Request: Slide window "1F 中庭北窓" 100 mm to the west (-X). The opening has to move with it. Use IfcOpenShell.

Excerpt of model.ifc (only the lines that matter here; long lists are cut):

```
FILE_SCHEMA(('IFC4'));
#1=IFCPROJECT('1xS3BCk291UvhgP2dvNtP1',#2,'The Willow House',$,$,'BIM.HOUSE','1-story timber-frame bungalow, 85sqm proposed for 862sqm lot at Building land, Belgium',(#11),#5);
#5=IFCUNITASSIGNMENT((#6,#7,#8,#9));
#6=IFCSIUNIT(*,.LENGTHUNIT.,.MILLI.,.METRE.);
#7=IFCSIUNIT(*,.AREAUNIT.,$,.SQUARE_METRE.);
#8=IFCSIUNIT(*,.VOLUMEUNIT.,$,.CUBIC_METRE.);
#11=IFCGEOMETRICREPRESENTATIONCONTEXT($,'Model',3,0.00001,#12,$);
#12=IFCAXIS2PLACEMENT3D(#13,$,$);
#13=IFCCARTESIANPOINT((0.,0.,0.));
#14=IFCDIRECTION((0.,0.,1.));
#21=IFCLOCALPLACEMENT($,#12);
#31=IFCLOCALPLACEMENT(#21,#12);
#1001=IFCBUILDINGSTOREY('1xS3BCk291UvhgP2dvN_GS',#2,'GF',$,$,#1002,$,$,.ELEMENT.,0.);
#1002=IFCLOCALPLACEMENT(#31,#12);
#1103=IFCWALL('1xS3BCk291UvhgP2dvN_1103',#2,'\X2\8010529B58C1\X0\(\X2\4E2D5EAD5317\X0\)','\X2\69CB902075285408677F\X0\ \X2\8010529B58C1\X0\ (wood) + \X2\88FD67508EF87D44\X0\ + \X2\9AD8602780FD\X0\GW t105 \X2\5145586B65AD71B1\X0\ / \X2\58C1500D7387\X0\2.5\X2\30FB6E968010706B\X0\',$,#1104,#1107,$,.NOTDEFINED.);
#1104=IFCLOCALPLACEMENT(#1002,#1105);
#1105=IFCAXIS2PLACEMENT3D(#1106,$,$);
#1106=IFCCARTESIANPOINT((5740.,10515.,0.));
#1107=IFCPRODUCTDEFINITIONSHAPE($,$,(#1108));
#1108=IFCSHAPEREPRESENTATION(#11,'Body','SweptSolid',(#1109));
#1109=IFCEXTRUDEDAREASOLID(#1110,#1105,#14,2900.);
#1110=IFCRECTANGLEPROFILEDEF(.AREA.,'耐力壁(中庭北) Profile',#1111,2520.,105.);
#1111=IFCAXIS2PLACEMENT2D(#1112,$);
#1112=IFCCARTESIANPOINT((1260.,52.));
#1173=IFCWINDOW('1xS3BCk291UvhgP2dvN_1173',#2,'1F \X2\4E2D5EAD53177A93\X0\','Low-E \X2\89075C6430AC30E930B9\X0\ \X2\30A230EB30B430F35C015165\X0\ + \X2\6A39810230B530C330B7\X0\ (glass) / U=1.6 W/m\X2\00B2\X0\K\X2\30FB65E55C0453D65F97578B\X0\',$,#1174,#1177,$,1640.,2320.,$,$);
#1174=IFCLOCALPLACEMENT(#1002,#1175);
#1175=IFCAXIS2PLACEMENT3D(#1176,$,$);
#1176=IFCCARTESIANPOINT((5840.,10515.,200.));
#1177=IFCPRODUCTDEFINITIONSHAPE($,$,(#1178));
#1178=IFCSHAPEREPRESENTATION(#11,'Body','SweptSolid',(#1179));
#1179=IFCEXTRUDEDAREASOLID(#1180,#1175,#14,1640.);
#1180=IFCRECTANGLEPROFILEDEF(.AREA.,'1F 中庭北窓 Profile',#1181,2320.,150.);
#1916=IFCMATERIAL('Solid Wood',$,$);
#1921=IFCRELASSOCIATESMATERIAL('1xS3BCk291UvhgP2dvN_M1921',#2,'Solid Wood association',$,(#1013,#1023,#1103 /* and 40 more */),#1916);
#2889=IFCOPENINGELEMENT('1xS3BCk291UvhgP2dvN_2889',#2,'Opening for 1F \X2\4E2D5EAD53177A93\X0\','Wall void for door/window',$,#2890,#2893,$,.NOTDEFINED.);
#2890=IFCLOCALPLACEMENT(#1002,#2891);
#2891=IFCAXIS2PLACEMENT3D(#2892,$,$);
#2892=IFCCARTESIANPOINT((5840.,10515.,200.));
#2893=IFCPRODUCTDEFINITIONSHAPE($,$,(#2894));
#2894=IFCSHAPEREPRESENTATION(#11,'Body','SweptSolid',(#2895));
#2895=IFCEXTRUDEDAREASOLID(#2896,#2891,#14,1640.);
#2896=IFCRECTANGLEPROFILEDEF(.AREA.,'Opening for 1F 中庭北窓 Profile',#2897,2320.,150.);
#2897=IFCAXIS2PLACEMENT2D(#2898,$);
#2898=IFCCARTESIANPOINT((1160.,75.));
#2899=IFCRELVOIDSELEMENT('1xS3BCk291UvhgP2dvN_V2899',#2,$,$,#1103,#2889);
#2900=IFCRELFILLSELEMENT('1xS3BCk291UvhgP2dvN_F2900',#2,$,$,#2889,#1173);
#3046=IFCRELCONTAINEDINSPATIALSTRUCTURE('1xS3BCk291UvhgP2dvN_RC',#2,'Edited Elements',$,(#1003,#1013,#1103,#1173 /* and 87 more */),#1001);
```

```python
import ifcopenshell
import ifcopenshell.api.geometry
import ifcopenshell.util.placement
import ifcopenshell.util.unit

model = ifcopenshell.open("model.ifc")
unit_scale = ifcopenshell.util.unit.calculate_unit_scale(model)

window = model.by_guid("1xS3BCk291UvhgP2dvN_1173")
opening = window.FillsVoids[0].RelatingOpeningElement
wall = opening.VoidsElements[0].RelatingBuildingElement

wall_matrix = ifcopenshell.util.placement.get_local_placement(wall.ObjectPlacement)
shift = wall_matrix[:3, 0] * -0.1 / unit_scale
before = ifcopenshell.util.placement.get_local_placement(window.ObjectPlacement)[:3, 3].copy()

# The window is not placed relative to its opening, so move both.
for product in (opening, window):
    matrix = ifcopenshell.util.placement.get_local_placement(product.ObjectPlacement)
    matrix[:3, 3] += shift
    ifcopenshell.api.geometry.edit_object_placement(model, product=product, matrix=matrix, is_si=False)

after = ifcopenshell.util.placement.get_local_placement(window.ObjectPlacement)[:3, 3]
print("window moved by", (after - before).round(3) + 0.0)

model.write("model_rev.ifc")
```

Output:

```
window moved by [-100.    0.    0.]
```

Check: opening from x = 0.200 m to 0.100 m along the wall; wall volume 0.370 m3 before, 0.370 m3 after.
